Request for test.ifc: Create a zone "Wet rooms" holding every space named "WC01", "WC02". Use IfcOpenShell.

First a look at what the model holds.

```python
import ifcopenshell

model = ifcopenshell.open("test.ifc")
print(model.schema)
seen = {}
for space in model.by_type("IfcSpace"):
    seen[space.LongName] = seen.get(space.LongName, 0) + 1
for name, count in sorted(seen.items(), key=str):
    print(count, "x", name)
print("zones:", [z.Name for z in model.by_type("IfcZone")][:20])
```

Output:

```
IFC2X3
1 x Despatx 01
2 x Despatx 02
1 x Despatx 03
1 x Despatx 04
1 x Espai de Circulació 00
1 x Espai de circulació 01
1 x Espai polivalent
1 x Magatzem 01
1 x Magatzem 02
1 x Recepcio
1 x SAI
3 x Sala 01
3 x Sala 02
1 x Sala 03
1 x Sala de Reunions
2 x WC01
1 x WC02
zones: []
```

```python
import ifcopenshell
import ifcopenshell.api.group
import ifcopenshell.api.root

model = ifcopenshell.open("test.ifc")

names = {"WC01", "WC02"}
spaces = [s for s in model.by_type("IfcSpace") if s.LongName in names]

zone = ifcopenshell.api.root.create_entity(model, ifc_class="IfcZone", name="Wet rooms")
ifcopenshell.api.group.assign_group(model, products=spaces, group=zone)
print(len(spaces), "spaces in", zone.Name)

model.write("test_v2.ifc")
```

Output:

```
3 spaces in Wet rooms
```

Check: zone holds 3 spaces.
